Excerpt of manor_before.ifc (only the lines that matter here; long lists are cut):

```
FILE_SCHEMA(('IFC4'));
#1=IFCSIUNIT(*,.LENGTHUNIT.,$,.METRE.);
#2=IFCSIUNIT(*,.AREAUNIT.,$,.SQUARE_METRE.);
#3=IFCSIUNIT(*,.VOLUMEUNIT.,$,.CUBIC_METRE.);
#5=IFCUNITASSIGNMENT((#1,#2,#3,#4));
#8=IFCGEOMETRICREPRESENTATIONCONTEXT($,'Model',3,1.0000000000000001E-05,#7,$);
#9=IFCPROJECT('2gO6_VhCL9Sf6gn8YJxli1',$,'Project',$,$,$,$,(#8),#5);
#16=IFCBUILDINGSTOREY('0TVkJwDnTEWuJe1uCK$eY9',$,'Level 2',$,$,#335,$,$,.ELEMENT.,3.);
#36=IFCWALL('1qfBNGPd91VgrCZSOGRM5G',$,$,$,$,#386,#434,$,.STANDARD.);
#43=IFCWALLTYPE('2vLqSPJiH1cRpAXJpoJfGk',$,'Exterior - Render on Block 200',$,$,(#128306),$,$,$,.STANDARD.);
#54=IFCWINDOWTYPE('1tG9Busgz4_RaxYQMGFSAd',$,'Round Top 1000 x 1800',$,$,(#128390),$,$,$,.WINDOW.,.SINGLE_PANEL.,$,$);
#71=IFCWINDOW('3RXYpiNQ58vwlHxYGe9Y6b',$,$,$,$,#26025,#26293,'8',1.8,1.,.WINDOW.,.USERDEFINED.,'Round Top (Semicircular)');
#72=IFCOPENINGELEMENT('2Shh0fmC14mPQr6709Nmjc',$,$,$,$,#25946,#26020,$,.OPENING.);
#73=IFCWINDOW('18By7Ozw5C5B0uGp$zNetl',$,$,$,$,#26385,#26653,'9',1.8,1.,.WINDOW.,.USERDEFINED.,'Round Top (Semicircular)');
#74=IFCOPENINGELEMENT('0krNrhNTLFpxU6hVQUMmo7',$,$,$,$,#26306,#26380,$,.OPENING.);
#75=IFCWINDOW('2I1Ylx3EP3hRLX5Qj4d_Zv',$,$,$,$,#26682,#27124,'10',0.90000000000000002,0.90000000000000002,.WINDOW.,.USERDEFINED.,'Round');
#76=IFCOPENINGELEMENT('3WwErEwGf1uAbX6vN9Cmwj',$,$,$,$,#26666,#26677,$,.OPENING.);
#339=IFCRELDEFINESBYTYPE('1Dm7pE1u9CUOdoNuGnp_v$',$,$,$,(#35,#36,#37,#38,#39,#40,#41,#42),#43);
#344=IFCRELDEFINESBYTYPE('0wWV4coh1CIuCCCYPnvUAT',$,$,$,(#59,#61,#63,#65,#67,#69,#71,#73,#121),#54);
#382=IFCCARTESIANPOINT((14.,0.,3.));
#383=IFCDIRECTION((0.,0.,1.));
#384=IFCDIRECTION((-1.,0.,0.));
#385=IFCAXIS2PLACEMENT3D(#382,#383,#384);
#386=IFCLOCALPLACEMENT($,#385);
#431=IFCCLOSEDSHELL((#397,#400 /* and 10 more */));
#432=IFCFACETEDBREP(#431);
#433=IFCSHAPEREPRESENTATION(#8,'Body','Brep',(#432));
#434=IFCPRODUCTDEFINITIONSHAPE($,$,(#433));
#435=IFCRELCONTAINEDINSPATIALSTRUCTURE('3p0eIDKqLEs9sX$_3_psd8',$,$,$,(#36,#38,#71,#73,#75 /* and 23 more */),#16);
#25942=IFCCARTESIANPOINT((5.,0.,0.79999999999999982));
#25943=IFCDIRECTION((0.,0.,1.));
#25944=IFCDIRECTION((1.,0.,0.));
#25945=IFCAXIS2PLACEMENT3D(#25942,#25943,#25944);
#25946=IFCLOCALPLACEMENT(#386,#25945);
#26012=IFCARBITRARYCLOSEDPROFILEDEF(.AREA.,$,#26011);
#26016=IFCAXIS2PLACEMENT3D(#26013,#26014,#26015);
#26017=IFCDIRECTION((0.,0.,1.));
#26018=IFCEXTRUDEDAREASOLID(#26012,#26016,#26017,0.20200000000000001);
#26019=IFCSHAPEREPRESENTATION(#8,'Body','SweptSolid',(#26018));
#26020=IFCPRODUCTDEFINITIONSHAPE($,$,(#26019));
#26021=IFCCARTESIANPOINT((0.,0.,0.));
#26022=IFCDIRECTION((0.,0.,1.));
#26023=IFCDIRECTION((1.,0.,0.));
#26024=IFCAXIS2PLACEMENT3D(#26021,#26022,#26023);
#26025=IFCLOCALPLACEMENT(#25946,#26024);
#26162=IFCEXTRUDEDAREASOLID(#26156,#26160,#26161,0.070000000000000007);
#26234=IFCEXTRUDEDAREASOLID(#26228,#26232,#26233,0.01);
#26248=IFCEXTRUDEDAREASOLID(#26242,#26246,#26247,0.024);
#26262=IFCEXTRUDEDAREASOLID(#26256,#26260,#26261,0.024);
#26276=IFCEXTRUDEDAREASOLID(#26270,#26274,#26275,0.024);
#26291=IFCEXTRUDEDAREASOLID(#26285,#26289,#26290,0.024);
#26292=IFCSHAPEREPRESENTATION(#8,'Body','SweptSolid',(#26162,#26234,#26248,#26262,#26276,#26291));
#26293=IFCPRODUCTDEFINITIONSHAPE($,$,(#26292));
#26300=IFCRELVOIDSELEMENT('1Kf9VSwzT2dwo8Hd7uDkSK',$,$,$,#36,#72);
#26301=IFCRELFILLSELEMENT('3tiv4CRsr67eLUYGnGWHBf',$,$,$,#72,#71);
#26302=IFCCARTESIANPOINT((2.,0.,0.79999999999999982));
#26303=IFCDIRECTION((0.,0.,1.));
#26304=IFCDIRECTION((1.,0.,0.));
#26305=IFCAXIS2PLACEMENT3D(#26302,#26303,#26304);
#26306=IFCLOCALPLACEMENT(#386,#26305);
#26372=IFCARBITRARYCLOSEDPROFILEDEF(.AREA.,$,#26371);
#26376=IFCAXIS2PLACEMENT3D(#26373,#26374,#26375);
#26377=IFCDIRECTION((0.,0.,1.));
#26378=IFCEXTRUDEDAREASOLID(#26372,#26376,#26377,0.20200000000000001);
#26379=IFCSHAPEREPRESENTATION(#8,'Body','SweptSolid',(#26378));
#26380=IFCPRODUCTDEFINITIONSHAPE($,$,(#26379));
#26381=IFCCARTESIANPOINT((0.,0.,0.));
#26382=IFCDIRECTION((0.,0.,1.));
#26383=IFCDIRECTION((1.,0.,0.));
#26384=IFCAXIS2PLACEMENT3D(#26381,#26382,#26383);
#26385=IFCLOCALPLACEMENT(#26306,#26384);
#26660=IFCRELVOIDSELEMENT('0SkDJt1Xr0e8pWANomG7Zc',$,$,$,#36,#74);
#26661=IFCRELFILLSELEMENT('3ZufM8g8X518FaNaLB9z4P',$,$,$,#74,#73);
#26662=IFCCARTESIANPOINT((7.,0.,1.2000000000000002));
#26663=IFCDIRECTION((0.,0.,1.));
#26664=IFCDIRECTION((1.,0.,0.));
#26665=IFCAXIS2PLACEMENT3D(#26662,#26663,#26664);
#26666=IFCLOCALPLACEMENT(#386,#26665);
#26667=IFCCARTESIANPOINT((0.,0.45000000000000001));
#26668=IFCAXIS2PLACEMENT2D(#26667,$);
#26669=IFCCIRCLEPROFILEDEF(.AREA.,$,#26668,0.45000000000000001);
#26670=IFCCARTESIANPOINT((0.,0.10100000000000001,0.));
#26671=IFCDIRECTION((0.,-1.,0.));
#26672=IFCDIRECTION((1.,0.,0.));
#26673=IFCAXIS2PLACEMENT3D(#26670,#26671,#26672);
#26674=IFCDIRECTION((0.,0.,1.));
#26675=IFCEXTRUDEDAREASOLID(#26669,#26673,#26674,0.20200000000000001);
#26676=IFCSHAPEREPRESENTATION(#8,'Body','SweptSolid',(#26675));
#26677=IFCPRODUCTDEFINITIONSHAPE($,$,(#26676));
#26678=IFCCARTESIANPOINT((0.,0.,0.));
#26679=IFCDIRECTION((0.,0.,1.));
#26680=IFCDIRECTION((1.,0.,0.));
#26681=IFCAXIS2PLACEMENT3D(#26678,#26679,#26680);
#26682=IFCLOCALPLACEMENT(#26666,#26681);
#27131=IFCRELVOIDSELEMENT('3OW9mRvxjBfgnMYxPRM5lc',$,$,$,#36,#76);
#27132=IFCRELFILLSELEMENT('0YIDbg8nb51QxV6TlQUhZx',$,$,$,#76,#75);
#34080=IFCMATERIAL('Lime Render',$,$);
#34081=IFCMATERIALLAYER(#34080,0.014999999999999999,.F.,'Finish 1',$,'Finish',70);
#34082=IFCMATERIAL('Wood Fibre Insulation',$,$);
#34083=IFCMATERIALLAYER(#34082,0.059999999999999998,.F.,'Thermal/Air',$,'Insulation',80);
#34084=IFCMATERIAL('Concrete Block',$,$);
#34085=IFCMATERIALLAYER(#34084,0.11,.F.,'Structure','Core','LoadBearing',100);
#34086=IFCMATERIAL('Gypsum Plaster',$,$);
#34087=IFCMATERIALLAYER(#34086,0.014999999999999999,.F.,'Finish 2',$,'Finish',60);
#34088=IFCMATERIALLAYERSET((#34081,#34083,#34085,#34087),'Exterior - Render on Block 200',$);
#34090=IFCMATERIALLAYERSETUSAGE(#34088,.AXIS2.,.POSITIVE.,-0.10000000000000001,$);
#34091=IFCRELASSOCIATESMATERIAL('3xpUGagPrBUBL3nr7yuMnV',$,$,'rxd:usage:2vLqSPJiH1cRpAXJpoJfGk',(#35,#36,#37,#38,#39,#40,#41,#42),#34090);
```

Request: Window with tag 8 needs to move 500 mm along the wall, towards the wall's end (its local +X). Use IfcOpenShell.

```python
import ifcopenshell
import ifcopenshell.api.geometry
import ifcopenshell.util.placement

model = ifcopenshell.open("manor_before.ifc")

window = model.by_guid("3RXYpiNQ58vwlHxYGe9Y6b")
opening = window.FillsVoids[0].RelatingOpeningElement
wall = opening.VoidsElements[0].RelatingBuildingElement

wall_matrix = ifcopenshell.util.placement.get_local_placement(wall.ObjectPlacement)
shift = wall_matrix[:3, 0] * 0.5
before = ifcopenshell.util.placement.get_local_placement(window.ObjectPlacement)[:3, 3].copy()

# The window is placed relative to its opening, so it follows when the opening moves.
matrix = ifcopenshell.util.placement.get_local_placement(opening.ObjectPlacement)
matrix[:3, 3] += shift
ifcopenshell.api.geometry.edit_object_placement(
    model, product=opening, matrix=matrix, is_si=False, should_transform_children=True
)

after = ifcopenshell.util.placement.get_local_placement(window.ObjectPlacement)[:3, 3]
print("window moved by", (after - before).round(3) + 0.0)

model.write("manor_before-out.ifc")
```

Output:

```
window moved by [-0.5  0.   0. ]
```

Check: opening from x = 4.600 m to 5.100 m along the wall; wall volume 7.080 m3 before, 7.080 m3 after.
